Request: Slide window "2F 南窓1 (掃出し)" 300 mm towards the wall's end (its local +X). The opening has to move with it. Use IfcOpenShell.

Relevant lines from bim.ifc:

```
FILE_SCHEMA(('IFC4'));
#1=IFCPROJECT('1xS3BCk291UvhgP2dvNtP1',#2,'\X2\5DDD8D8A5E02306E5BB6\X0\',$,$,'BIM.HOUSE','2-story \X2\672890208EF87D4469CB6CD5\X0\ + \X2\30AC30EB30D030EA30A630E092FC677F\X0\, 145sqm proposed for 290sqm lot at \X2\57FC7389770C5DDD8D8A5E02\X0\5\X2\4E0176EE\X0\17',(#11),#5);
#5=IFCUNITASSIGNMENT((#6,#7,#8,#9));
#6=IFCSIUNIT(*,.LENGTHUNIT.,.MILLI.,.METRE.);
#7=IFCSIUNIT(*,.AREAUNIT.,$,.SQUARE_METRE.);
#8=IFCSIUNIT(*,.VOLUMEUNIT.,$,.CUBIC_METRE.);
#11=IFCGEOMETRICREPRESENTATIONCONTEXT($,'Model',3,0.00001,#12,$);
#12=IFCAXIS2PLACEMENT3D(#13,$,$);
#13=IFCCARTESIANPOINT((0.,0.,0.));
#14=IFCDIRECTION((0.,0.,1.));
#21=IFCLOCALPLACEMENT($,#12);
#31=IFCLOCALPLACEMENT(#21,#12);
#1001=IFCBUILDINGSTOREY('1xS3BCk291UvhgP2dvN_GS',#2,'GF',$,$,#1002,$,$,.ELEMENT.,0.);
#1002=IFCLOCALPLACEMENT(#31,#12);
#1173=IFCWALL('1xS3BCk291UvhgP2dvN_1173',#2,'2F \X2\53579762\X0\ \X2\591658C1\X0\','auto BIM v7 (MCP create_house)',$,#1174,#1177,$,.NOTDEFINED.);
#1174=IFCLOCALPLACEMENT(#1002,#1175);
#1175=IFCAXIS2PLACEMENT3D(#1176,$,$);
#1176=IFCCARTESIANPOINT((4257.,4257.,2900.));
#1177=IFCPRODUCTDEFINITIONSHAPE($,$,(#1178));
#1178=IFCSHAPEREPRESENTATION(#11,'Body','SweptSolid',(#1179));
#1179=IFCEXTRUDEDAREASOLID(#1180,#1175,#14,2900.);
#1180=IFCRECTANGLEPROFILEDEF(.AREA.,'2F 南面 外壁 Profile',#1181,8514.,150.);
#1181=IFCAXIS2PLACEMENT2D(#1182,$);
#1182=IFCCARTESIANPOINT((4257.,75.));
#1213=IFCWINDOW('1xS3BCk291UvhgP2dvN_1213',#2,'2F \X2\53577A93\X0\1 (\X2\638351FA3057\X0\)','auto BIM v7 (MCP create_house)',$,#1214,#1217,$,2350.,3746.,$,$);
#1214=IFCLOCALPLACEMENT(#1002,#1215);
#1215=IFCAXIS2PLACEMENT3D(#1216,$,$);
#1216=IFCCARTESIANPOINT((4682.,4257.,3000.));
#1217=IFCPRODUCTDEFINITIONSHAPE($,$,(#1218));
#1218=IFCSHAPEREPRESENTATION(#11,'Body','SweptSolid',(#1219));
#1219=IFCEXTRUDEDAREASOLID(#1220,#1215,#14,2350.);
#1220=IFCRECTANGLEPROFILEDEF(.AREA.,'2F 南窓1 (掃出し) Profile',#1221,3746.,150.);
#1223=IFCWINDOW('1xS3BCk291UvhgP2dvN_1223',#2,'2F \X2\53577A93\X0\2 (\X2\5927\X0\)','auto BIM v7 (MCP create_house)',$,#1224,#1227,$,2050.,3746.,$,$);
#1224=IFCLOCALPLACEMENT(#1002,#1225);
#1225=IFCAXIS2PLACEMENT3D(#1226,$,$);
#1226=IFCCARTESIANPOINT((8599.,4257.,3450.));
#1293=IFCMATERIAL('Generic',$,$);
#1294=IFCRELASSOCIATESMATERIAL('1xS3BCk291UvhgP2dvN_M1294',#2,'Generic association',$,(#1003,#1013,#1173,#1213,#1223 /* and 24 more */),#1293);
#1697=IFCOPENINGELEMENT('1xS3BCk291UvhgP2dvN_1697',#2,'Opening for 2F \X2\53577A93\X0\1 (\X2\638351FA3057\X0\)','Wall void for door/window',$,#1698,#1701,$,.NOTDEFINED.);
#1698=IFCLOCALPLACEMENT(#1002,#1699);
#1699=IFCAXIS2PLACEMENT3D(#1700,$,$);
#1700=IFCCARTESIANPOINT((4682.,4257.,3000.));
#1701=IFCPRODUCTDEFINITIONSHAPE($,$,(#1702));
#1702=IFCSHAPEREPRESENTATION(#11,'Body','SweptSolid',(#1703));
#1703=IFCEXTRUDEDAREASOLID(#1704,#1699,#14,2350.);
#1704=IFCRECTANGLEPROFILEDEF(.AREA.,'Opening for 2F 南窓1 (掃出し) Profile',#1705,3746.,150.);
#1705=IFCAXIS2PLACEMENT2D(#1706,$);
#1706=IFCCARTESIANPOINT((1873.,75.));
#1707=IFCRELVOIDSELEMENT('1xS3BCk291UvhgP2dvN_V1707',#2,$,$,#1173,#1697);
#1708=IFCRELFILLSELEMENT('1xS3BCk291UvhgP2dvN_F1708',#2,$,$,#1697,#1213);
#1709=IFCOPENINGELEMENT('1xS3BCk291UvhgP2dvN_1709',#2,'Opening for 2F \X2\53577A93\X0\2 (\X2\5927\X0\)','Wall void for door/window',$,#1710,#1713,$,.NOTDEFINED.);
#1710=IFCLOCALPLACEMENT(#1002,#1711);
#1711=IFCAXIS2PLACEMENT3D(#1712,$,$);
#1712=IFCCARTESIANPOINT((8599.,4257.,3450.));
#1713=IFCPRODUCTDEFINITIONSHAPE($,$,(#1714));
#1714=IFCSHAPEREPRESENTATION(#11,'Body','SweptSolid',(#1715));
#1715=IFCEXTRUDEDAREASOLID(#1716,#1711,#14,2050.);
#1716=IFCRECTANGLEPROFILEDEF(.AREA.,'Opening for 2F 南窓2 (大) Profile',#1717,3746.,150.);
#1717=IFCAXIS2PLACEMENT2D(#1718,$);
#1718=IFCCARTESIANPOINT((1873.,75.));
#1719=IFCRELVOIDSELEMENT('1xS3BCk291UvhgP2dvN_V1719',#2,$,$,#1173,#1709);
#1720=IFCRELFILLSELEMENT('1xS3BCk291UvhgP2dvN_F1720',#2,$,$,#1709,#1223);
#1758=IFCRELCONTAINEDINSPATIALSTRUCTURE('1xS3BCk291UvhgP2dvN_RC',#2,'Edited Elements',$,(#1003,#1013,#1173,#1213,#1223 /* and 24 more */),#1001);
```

```python
import ifcopenshell
import ifcopenshell.api.geometry
import ifcopenshell.util.placement

model = ifcopenshell.open("bim.ifc")

window = model.by_guid("1xS3BCk291UvhgP2dvN_1213")
opening = window.FillsVoids[0].RelatingOpeningElement
wall = opening.VoidsElements[0].RelatingBuildingElement

wall_matrix = ifcopenshell.util.placement.get_local_placement(wall.ObjectPlacement)
shift = wall_matrix[:3, 0] * 300.0
before = ifcopenshell.util.placement.get_local_placement(window.ObjectPlacement)[:3, 3].copy()

# The window is not placed relative to its opening, so move both.
for product in (opening, window):
    matrix = ifcopenshell.util.placement.get_local_placement(product.ObjectPlacement)
    matrix[:3, 3] += shift
    ifcopenshell.api.geometry.edit_object_placement(model, product=product, matrix=matrix, is_si=False)

after = ifcopenshell.util.placement.get_local_placement(window.ObjectPlacement)[:3, 3]
print("window moved by", (after - before).round(3) + 0.0)

model.write("bim_rev.ifc")
```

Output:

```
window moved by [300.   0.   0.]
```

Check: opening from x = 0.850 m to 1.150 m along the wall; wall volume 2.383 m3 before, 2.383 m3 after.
